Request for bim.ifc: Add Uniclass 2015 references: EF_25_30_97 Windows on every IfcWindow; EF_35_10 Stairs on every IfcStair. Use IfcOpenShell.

First a look at what the model holds.

```python
import ifcopenshell

model = ifcopenshell.open("bim.ifc")
print(model.schema)
print("classifications:", [c.Name for c in model.by_type("IfcClassification")])
for ifc_class in ("IfcDoor", "IfcRoof", "IfcStair", "IfcWall", "IfcWindow"):
    print(ifc_class, len(model.by_type(ifc_class)))
```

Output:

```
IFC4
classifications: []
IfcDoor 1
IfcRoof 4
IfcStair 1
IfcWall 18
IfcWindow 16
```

```python
import ifcopenshell
import ifcopenshell.api.classification

model = ifcopenshell.open("bim.ifc")

system = ifcopenshell.api.classification.add_classification(model, classification="Uniclass 2015")

codes = {
    "IfcWindow": ("EF_25_30_97", "Windows"),
    "IfcStair": ("EF_35_10", "Stairs"),
}
for ifc_class, (code, name) in codes.items():
    products = model.by_type(ifc_class)
    ifcopenshell.api.classification.add_reference(
        model, products=products, classification=system, identification=code, name=name
    )
    print(code, len(products))

model.write("bim_updated.ifc")
```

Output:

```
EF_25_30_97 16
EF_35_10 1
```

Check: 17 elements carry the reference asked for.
